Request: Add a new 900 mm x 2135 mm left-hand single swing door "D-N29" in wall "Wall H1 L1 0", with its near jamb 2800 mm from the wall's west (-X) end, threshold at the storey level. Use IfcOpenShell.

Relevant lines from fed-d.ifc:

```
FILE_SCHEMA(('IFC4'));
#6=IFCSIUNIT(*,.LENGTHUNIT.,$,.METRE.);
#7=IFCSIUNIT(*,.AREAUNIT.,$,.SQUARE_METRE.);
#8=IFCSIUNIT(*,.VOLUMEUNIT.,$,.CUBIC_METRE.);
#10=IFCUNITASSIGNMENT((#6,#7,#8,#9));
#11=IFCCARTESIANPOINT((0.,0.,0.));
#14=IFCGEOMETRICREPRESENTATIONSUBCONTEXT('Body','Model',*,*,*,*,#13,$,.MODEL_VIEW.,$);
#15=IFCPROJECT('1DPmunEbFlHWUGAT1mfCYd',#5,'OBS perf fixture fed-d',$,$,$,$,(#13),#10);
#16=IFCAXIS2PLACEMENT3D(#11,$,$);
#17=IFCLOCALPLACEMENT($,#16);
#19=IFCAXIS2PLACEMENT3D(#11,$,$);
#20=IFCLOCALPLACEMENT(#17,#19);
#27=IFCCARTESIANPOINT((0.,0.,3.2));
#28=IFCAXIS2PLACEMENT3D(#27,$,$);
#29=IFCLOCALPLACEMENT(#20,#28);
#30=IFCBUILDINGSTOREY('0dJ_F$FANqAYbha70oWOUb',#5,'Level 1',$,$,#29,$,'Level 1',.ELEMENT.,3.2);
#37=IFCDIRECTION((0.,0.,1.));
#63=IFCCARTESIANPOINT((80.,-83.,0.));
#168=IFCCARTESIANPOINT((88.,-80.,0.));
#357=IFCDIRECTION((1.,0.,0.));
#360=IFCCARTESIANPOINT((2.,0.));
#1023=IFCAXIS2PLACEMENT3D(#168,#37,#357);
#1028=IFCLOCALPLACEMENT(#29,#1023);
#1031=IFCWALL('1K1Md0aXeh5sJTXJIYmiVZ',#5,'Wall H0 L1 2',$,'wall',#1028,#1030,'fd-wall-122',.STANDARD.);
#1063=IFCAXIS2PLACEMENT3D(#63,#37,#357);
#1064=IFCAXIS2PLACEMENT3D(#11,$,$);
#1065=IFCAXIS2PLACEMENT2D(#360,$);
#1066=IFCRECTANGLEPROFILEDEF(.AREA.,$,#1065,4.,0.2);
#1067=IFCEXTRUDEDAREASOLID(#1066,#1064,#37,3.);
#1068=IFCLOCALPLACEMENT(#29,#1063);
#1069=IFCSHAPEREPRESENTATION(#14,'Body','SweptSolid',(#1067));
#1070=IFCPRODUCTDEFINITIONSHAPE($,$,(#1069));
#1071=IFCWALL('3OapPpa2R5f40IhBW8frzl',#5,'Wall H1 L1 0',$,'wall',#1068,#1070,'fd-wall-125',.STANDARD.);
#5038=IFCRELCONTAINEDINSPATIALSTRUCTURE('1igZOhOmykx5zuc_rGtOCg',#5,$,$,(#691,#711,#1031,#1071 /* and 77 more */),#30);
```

```python
import numpy as np
import ifcopenshell
import ifcopenshell.api.feature
import ifcopenshell.api.geometry
import ifcopenshell.api.root
import ifcopenshell.api.spatial
import ifcopenshell.geom
import ifcopenshell.util.element
import ifcopenshell.util.placement
import ifcopenshell.util.representation
import ifcopenshell.util.shape
import ifcopenshell.util.unit

model = ifcopenshell.open("fed-d.ifc")
unit_scale = ifcopenshell.util.unit.calculate_unit_scale(model)
settings = ifcopenshell.geom.settings()


def volume(element):
    """Net volume in cubic metres, openings subtracted."""
    shape = ifcopenshell.geom.create_shape(settings, element)
    return ifcopenshell.util.shape.get_volume(shape.geometry)


wall = model.by_guid("3OapPpa2R5f40IhBW8frzl")
storey = ifcopenshell.util.element.get_container(wall, ifc_class="IfcBuildingStorey")
context = ifcopenshell.util.representation.get_context(model, "Model", "Body", "MODEL_VIEW")
before = volume(wall)

width, height, from_end, sill = 0.9, 2.135, 2.8, 0.0  # metres

# The wall runs along its own X axis, and the end named is its -X end.
wall_shape = ifcopenshell.geom.create_shape(settings, wall)
x, y, z = ifcopenshell.util.shape.get_vertices(wall_shape.geometry).T
start = x.min() + from_end
face, thickness = float(y.min()), float(y.max() - y.min())
wall_matrix = ifcopenshell.util.placement.get_local_placement(wall.ObjectPlacement)
level = ifcopenshell.util.placement.get_local_placement(storey.ObjectPlacement)[2, 3]


def in_wall(x, y):
    """Placement at x, y metres in the wall's axes, at sill height."""
    matrix = wall_matrix.copy()
    matrix[:, 3] = wall_matrix @ np.array([x / unit_scale, y / unit_scale, 0.0, 1.0])
    matrix[2, 3] = level + sill / unit_scale
    return matrix


# Opening: a box that overshoots both wall faces by 50 mm.
opening = ifcopenshell.api.root.create_entity(model, ifc_class="IfcOpeningElement", predefined_type="OPENING")
box = ifcopenshell.api.geometry.add_wall_representation(
    model, context=context, length=width, height=height, thickness=thickness + 0.1
)
ifcopenshell.api.geometry.assign_representation(model, product=opening, representation=box)
ifcopenshell.api.geometry.edit_object_placement(model, product=opening, matrix=in_wall(start, face - 0.05), is_si=False)
ifcopenshell.api.feature.add_feature(model, feature=opening, element=wall)

door = ifcopenshell.api.root.create_entity(model, ifc_class="IfcDoor", name="D-N29", predefined_type="DOOR")
door.OverallWidth, door.OverallHeight = width / unit_scale, height / unit_scale
door.OperationType = "SINGLE_SWING_LEFT"
body = ifcopenshell.api.geometry.add_door_representation(
    model,
    context=context,
    overall_width=door.OverallWidth,
    overall_height=door.OverallHeight,
    operation_type="SINGLE_SWING_LEFT",
    lining_properties={"LiningDepth": thickness / unit_scale, "ThresholdDepth": thickness / unit_scale},
)
ifcopenshell.api.geometry.assign_representation(model, product=door, representation=body)
ifcopenshell.api.spatial.assign_container(model, products=[door], relating_structure=storey)
ifcopenshell.api.feature.add_filling(model, opening=opening, element=door)

# The lining spans the wall, so the door starts at the wall face.
ifcopenshell.api.geometry.edit_object_placement(model, product=door, matrix=in_wall(start, face), is_si=False)

after = volume(wall)

print(f"wall volume {before:.3f} -> {after:.3f} m3")

model.write("fed-d_rev.ifc")
```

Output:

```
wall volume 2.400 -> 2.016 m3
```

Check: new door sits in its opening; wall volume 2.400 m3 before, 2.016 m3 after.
